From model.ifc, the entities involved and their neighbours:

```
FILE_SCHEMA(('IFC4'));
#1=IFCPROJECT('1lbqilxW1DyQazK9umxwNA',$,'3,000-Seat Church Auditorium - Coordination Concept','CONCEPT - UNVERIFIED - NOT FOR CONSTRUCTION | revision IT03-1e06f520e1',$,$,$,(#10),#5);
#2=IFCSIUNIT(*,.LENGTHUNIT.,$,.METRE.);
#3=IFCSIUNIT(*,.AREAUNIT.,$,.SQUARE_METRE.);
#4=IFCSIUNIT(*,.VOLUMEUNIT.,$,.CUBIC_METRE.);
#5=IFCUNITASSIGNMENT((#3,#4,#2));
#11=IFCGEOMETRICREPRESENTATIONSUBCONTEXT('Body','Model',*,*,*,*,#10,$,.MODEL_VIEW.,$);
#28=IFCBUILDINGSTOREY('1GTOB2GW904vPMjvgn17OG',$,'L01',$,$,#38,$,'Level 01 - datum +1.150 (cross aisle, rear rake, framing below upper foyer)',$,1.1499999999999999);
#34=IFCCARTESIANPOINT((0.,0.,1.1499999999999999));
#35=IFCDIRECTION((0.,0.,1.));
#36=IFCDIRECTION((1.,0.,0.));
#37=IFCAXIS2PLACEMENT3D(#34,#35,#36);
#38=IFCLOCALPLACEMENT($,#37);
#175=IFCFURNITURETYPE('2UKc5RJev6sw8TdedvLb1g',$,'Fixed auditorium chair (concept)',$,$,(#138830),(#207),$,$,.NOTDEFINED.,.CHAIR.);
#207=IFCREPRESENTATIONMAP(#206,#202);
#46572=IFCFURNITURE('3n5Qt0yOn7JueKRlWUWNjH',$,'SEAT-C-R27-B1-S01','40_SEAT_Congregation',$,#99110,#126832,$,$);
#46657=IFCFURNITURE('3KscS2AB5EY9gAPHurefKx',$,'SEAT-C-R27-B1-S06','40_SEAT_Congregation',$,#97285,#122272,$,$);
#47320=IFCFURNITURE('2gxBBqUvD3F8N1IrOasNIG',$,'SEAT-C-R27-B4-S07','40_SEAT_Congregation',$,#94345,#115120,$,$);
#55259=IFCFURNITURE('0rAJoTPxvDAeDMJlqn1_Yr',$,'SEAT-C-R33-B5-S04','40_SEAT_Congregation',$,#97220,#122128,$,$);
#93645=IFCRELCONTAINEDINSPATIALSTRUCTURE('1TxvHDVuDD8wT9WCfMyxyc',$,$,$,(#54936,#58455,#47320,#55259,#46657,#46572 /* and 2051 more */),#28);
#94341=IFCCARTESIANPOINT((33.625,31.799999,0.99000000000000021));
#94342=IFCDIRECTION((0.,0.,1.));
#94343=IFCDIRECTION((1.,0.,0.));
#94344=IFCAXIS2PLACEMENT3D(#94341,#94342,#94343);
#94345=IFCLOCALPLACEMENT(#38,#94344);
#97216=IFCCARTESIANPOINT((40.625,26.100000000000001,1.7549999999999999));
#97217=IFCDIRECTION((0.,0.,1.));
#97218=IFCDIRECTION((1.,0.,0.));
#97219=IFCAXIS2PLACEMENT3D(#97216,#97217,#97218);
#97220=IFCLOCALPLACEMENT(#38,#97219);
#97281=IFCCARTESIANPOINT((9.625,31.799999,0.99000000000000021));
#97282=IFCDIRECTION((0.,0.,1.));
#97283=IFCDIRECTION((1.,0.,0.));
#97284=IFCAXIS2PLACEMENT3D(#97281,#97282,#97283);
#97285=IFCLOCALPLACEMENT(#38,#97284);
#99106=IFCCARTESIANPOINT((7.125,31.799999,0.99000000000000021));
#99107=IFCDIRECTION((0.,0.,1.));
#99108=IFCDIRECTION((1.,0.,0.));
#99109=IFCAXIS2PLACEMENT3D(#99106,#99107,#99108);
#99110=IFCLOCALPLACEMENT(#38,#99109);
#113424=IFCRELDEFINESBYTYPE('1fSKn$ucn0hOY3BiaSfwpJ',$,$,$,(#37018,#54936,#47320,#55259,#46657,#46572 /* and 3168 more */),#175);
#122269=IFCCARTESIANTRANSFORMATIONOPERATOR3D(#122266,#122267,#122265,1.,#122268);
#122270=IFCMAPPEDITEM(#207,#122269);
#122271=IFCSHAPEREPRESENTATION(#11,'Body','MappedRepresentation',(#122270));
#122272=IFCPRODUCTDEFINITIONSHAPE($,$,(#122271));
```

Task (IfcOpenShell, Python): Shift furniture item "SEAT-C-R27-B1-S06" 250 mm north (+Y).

```python
import ifcopenshell
import ifcopenshell.api.geometry
import ifcopenshell.util.placement

model = ifcopenshell.open("model.ifc")

item = model.by_id(46657)
matrix = ifcopenshell.util.placement.get_local_placement(item.ObjectPlacement)
matrix[1, 3] += 0.25
ifcopenshell.api.geometry.edit_object_placement(model, product=item, matrix=matrix, is_si=False)

print(ifcopenshell.util.placement.get_local_placement(item.ObjectPlacement).round(3) + 0.0)

model.write("model-out.ifc")
```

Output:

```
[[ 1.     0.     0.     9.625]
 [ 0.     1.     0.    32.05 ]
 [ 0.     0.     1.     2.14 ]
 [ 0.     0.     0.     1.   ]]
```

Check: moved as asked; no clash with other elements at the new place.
